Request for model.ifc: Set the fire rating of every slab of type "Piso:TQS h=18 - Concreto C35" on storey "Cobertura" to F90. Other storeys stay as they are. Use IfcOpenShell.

First a look at what the model holds.

```python
import ifcopenshell
import ifcopenshell.util.element

model = ifcopenshell.open("model.ifc")
print(model.schema)
storey = next(s for s in model.by_type("IfcBuildingStorey") if s.Name == "Cobertura")
slabs = [e for e in ifcopenshell.util.element.get_decomposition(storey) if e.is_a("IfcSlab")]
seen = {}
for e in slabs:
    element_type = ifcopenshell.util.element.get_type(e)
    key = (element_type.Name if element_type != e and element_type else None, ifcopenshell.util.element.get_pset(e, "Pset_SlabCommon", "FireRating"))
    seen[key] = seen.get(key, 0) + 1
for (name, value), count in sorted(seen.items(), key=str):
    print(count, "x", name, "|", value)
```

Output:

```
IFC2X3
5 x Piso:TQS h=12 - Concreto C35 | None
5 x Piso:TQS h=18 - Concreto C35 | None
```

```python
import ifcopenshell
import ifcopenshell.api.pset
import ifcopenshell.util.element

model = ifcopenshell.open("model.ifc")

storey = next(s for s in model.by_type("IfcBuildingStorey") if s.Name == "Cobertura")
slabs = [e for e in ifcopenshell.util.element.get_decomposition(storey) if e.is_a("IfcSlab")]

count = 0
for e in slabs:
    element_type = ifcopenshell.util.element.get_type(e)
    if element_type in (None, e) or element_type.Name != "Piso:TQS h=18 - Concreto C35":
        continue
    # add_pset returns the element's existing set when there is one.
    pset = ifcopenshell.api.pset.add_pset(model, product=e, name="Pset_SlabCommon")
    ifcopenshell.api.pset.edit_pset(model, pset=pset, properties={"FireRating": "F90"})
    count += 1

print(count, "slabs updated")

model.write("model_v2.ifc")
```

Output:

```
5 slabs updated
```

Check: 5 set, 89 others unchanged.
